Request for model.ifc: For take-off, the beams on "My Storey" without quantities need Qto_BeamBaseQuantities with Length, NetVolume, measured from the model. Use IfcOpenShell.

First a look at what the model holds.

```python
import ifcopenshell
import ifcopenshell.util.element
import ifcopenshell.util.unit

model = ifcopenshell.open("model.ifc")
print(model.schema)
for unit_type in ("LENGTHUNIT", "AREAUNIT", "VOLUMEUNIT"):
    print(unit_type, ifcopenshell.util.unit.calculate_unit_scale(model, unit_type))
storey = next(s for s in model.by_type("IfcBuildingStorey") if s.Name == "My Storey")
beams = [e for e in ifcopenshell.util.element.get_decomposition(storey) if e.is_a("IfcBeam")]
for e in sorted(beams, key=lambda e: e.id()):
    print(e.id(), e.is_a(), e.Name, list(ifcopenshell.util.element.get_psets(e, qtos_only=True)), sep=" | ")
```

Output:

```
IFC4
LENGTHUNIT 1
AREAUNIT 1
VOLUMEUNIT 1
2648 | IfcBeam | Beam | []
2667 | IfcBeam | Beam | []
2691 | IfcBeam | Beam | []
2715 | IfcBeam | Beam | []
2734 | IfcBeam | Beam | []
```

```python
import ifcopenshell
import ifcopenshell.api.pset
import ifcopenshell.geom
import ifcopenshell.util.element
import ifcopenshell.util.shape
import ifcopenshell.util.unit

model = ifcopenshell.open("model.ifc")
unit_scale = ifcopenshell.util.unit.calculate_unit_scale(model)
volume_scale = ifcopenshell.util.unit.calculate_unit_scale(model, "VOLUMEUNIT")
settings = ifcopenshell.geom.settings()

storey = next(s for s in model.by_type("IfcBuildingStorey") if s.Name == "My Storey")
beams = [e for e in ifcopenshell.util.element.get_decomposition(storey) if e.is_a("IfcBeam")]

for e in sorted(beams, key=lambda e: e.id()):
    if ifcopenshell.util.element.get_psets(e, qtos_only=True, should_inherit=False):
        continue
    # Geometry comes back in metres, in the element's own axes.
    shape = ifcopenshell.geom.create_shape(settings, e)
    values = {
        "Length": ifcopenshell.util.shape.get_max_xyz(shape.geometry) / unit_scale,
        "NetVolume": ifcopenshell.util.shape.get_volume(shape.geometry) / volume_scale,
    }
    qto = ifcopenshell.api.pset.add_qto(model, product=e, name="Qto_BeamBaseQuantities")
    ifcopenshell.api.pset.edit_qto(model, qto=qto, properties=values)
    print(e.id(), {k: round(v, 3) for k, v in values.items()})

model.write("model_rev.ifc")
```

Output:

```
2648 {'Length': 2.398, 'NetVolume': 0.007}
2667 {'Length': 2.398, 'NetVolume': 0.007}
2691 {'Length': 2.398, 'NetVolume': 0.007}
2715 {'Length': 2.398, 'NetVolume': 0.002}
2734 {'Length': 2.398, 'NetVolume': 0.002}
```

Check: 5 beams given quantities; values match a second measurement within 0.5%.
